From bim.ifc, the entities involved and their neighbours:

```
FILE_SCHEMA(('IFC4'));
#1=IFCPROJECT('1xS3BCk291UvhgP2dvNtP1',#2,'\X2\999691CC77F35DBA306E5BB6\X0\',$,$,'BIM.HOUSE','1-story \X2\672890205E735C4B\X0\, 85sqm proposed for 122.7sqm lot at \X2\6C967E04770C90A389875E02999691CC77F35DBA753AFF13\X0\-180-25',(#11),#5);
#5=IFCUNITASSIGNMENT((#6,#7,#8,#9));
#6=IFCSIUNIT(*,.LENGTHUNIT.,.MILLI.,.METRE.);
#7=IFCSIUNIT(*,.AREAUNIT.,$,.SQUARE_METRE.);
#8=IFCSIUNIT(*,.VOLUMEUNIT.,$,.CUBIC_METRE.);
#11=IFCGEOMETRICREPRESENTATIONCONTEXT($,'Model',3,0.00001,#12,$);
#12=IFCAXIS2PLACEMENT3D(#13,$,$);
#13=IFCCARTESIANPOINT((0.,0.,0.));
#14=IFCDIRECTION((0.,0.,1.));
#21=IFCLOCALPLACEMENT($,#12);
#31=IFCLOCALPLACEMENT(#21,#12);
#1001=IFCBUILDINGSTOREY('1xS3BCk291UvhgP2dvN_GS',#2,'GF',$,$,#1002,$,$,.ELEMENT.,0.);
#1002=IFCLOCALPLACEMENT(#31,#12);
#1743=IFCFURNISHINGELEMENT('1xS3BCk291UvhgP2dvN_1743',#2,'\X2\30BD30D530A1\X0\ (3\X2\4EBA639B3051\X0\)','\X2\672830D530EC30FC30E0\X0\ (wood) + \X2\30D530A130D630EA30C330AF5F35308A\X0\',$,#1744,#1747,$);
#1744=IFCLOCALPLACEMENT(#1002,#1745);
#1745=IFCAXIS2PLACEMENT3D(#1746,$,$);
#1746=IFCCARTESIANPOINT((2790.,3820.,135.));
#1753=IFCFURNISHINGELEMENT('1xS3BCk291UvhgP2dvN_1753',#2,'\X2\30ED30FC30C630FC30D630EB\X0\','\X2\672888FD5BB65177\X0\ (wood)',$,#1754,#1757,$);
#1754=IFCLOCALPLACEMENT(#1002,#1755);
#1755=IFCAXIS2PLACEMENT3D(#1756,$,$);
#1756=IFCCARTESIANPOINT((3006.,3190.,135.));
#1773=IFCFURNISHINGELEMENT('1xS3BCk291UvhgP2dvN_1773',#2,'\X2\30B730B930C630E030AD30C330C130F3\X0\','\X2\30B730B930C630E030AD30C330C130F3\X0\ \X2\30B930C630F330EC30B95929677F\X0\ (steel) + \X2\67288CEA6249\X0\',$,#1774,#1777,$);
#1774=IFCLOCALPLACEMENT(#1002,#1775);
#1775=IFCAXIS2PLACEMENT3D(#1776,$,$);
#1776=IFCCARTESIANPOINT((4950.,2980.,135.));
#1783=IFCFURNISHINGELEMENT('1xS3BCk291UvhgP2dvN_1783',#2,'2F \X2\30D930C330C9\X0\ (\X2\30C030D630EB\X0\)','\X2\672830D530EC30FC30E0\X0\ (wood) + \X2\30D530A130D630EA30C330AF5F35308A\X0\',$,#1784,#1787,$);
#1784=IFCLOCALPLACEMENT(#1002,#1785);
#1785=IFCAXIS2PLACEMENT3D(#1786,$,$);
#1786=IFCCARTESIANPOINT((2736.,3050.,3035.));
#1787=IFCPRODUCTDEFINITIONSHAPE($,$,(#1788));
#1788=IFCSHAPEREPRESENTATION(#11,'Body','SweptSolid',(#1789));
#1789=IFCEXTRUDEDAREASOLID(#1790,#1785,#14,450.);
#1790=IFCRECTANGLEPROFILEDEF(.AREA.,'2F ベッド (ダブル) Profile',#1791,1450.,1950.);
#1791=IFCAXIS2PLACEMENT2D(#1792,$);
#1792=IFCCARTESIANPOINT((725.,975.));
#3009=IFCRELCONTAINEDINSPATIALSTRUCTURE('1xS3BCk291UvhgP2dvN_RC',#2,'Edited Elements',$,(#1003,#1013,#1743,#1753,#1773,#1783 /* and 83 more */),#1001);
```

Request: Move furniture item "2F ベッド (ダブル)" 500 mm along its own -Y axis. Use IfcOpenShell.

```python
import ifcopenshell
import ifcopenshell.api.geometry
import ifcopenshell.util.placement

model = ifcopenshell.open("bim.ifc")

item = model.by_guid("1xS3BCk291UvhgP2dvN_1783")
matrix = ifcopenshell.util.placement.get_local_placement(item.ObjectPlacement)
matrix[:3, 3] -= matrix[:3, 1] * 500.0
ifcopenshell.api.geometry.edit_object_placement(model, product=item, matrix=matrix, is_si=False)

print(ifcopenshell.util.placement.get_local_placement(item.ObjectPlacement).round(3) + 0.0)

model.write("bim-out.ifc")
```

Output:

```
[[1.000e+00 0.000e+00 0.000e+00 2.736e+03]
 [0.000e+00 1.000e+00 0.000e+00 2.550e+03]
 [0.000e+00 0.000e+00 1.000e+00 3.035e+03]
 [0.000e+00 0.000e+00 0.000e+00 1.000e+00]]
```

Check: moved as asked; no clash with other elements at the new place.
